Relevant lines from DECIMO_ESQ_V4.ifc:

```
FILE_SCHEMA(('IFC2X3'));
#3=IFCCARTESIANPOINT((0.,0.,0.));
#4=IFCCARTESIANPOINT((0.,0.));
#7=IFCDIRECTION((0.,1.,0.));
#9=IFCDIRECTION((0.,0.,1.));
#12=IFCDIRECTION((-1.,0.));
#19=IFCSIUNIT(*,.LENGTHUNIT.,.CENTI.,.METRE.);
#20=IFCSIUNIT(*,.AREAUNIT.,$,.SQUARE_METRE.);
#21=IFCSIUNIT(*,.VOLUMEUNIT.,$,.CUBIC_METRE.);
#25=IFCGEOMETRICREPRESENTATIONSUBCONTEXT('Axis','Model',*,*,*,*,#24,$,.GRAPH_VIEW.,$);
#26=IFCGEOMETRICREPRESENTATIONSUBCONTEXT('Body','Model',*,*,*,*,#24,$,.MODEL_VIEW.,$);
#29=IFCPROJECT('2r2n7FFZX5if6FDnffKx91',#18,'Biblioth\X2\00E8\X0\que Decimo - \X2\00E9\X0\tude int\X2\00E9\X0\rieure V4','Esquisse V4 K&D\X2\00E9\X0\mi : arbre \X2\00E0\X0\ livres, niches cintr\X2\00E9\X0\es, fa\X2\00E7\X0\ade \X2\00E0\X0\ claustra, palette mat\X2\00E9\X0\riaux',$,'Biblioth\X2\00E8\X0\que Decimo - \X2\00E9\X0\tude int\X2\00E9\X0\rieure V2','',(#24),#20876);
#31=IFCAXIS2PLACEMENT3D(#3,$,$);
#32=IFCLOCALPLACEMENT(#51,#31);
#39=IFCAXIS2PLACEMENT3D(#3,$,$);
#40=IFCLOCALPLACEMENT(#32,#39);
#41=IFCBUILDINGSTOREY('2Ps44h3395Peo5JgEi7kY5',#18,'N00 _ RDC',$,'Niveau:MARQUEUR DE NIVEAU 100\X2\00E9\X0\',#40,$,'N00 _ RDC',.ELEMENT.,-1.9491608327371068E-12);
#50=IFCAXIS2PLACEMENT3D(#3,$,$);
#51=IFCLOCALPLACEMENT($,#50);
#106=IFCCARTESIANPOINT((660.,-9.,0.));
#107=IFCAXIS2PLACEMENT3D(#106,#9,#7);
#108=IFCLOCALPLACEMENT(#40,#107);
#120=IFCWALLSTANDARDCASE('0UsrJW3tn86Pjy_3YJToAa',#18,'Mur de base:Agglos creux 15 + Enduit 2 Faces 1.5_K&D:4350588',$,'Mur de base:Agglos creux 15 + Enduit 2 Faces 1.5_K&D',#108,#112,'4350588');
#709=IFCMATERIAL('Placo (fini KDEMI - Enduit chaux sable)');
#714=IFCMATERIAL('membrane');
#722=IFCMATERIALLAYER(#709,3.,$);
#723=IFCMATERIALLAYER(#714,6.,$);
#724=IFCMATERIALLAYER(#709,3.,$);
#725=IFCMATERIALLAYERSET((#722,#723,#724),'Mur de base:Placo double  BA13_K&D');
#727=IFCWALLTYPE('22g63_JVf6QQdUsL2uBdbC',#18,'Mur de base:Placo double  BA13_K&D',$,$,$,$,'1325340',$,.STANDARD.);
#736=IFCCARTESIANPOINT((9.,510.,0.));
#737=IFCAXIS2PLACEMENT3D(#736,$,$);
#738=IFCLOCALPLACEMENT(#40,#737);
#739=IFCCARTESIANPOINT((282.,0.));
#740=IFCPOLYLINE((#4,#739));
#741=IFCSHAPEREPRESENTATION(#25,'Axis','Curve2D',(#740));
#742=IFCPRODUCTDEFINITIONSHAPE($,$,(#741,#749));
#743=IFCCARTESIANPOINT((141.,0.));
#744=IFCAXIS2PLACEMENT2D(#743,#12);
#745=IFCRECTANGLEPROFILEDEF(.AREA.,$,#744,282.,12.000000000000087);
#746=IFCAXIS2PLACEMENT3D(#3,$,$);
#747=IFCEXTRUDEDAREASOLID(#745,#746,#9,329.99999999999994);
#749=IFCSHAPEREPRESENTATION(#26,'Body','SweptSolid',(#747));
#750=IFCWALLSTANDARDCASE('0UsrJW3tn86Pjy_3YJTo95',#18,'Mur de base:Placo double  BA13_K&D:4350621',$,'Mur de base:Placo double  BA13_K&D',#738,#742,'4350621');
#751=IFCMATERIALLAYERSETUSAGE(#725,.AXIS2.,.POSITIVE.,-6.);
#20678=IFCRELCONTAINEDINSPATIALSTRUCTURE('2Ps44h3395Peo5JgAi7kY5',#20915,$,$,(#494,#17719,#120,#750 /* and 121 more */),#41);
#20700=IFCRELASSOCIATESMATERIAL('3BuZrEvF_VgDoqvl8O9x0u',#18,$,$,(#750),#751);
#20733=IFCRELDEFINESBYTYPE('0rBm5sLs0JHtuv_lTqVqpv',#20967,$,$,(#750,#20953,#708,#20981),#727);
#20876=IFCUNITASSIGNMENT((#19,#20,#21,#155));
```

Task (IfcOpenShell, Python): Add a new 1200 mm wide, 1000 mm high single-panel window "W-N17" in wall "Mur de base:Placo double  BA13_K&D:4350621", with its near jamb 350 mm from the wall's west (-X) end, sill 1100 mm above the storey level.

```python
import numpy as np
import ifcopenshell
import ifcopenshell.api.feature
import ifcopenshell.api.geometry
import ifcopenshell.api.root
import ifcopenshell.api.spatial
import ifcopenshell.api.type
import ifcopenshell.geom
import ifcopenshell.util.element
import ifcopenshell.util.placement
import ifcopenshell.util.representation
import ifcopenshell.util.shape
import ifcopenshell.util.unit

model = ifcopenshell.open("DECIMO_ESQ_V4.ifc")
unit_scale = ifcopenshell.util.unit.calculate_unit_scale(model)
settings = ifcopenshell.geom.settings()


def volume(element):
    """Net volume in cubic metres, openings subtracted."""
    shape = ifcopenshell.geom.create_shape(settings, element)
    return ifcopenshell.util.shape.get_volume(shape.geometry)


wall = model.by_guid("0UsrJW3tn86Pjy_3YJTo95")
storey = ifcopenshell.util.element.get_container(wall, ifc_class="IfcBuildingStorey")
context = ifcopenshell.util.representation.get_context(model, "Model", "Body", "MODEL_VIEW")
before = volume(wall)

width, height, from_end, sill = 1.2, 1, 0.35, 1.1  # metres

# The wall runs along its own X axis, and the end named is its -X end.
wall_shape = ifcopenshell.geom.create_shape(settings, wall)
x, y, z = ifcopenshell.util.shape.get_vertices(wall_shape.geometry).T
start = x.min() + from_end
face, thickness = float(y.min()), float(y.max() - y.min())
wall_matrix = ifcopenshell.util.placement.get_local_placement(wall.ObjectPlacement)
level = ifcopenshell.util.placement.get_local_placement(storey.ObjectPlacement)[2, 3]


def in_wall(x, y):
    """Placement at x, y metres in the wall's axes, at sill height."""
    matrix = wall_matrix.copy()
    matrix[:, 3] = wall_matrix @ np.array([x / unit_scale, y / unit_scale, 0.0, 1.0])
    matrix[2, 3] = level + sill / unit_scale
    return matrix


# Opening: a box that overshoots both wall faces by 50 mm.
opening = ifcopenshell.api.root.create_entity(model, ifc_class="IfcOpeningElement")
box = ifcopenshell.api.geometry.add_wall_representation(
    model, context=context, length=width, height=height, thickness=thickness + 0.1
)
ifcopenshell.api.geometry.assign_representation(model, product=opening, representation=box)
ifcopenshell.api.geometry.edit_object_placement(model, product=opening, matrix=in_wall(start, face - 0.05), is_si=False)
ifcopenshell.api.feature.add_feature(model, feature=opening, element=wall)

window = ifcopenshell.api.root.create_entity(model, ifc_class="IfcWindow", name="W-N17")
window.OverallWidth, window.OverallHeight = width / unit_scale, height / unit_scale
body = ifcopenshell.api.geometry.add_window_representation(
    model,
    context=context,
    overall_width=window.OverallWidth,
    overall_height=window.OverallHeight,
    partition_type="SINGLE_PANEL",
)
ifcopenshell.api.geometry.assign_representation(model, product=window, representation=body)
ifcopenshell.api.spatial.assign_container(model, products=[window], relating_structure=storey)
fills = ifcopenshell.api.feature.add_filling(model, opening=opening, element=window)
fills.OwnerHistory = window.OwnerHistory  # required in IFC2X3

# IFC2X3 keeps the operation on the window style.
style = ifcopenshell.api.root.create_entity(model, ifc_class="IfcWindowStyle", name="W-N17")
style.OperationType, style.ConstructionType = "SINGLE_PANEL", "NOTDEFINED"
style.ParameterTakesPrecedence = style.Sizeable = False
ifcopenshell.api.type.assign_type(model, related_objects=[window], relating_type=style)

# Centre the window in the wall's thickness.
ifcopenshell.api.geometry.edit_object_placement(model, product=window, matrix=in_wall(start, face), is_si=False)
window_shape = ifcopenshell.geom.create_shape(settings, window)
depth = ifcopenshell.util.shape.get_vertices(window_shape.geometry)[:, 1]
offset = face + thickness / 2 - (depth.min() + depth.max()) / 2
ifcopenshell.api.geometry.edit_object_placement(model, product=window, matrix=in_wall(start, offset), is_si=False)

after = volume(wall)

print(f"wall volume {before:.3f} -> {after:.3f} m3")

model.write("DECIMO_ESQ_V4_updated.ifc")
```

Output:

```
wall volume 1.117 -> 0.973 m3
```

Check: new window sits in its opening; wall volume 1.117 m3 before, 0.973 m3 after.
